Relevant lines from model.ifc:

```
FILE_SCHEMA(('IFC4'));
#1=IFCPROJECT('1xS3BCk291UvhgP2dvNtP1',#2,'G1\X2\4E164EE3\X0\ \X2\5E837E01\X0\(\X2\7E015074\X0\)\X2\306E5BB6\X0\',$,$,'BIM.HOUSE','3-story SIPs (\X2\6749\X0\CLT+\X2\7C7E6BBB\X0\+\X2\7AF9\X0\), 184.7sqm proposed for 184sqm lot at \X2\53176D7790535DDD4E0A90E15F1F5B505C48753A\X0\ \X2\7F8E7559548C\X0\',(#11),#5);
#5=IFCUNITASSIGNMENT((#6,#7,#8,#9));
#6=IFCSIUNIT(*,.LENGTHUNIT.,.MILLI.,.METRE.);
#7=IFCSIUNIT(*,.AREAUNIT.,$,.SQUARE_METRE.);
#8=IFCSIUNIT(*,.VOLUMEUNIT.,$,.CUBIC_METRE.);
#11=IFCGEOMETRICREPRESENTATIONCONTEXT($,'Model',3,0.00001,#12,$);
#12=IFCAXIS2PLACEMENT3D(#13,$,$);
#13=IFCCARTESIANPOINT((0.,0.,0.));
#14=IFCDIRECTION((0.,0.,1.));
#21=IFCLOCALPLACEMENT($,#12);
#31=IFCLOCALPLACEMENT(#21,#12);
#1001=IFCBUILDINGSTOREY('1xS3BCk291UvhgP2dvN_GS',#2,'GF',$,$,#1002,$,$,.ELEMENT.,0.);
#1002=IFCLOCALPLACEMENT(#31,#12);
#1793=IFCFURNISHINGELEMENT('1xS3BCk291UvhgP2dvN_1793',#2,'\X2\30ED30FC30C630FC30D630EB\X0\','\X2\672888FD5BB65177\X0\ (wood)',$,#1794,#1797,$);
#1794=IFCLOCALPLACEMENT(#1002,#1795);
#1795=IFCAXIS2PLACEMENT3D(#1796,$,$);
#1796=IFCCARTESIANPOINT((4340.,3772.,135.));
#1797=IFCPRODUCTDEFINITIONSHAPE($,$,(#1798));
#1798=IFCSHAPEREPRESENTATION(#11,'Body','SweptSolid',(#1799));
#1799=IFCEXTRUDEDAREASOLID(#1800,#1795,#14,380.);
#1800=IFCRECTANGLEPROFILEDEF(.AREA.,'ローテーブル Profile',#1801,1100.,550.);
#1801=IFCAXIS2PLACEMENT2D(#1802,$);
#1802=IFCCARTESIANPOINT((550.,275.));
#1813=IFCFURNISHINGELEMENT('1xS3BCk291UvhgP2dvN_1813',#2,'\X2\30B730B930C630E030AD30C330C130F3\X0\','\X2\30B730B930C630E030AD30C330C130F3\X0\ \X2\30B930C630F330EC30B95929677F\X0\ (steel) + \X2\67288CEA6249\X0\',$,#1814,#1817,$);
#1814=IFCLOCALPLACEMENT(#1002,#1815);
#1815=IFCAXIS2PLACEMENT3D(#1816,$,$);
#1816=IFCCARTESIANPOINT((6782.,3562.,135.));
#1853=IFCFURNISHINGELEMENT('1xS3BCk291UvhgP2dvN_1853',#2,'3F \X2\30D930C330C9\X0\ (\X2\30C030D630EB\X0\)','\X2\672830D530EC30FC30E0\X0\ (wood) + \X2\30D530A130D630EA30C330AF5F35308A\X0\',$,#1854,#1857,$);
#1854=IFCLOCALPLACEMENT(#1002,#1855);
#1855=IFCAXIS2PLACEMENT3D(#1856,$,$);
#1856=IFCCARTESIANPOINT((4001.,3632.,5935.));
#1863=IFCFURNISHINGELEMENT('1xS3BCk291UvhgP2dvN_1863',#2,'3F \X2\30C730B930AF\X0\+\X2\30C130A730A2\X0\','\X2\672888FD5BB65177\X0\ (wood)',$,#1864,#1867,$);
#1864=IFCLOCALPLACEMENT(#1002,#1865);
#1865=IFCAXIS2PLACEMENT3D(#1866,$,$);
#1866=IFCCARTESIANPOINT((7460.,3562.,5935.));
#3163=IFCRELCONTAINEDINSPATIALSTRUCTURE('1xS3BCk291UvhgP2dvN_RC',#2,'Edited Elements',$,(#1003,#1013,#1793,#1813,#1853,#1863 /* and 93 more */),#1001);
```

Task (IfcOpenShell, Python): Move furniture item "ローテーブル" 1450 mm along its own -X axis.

```python
import ifcopenshell
import ifcopenshell.api.geometry
import ifcopenshell.util.placement
import ifcopenshell.util.unit

model = ifcopenshell.open("model.ifc")
unit_scale = ifcopenshell.util.unit.calculate_unit_scale(model)

item = model.by_guid("1xS3BCk291UvhgP2dvN_1793")
matrix = ifcopenshell.util.placement.get_local_placement(item.ObjectPlacement)
matrix[:3, 3] -= matrix[:3, 0] * 1.45 / unit_scale
ifcopenshell.api.geometry.edit_object_placement(model, product=item, matrix=matrix, is_si=False)

print(ifcopenshell.util.placement.get_local_placement(item.ObjectPlacement).round(3) + 0.0)

model.write("model_rev.ifc")
```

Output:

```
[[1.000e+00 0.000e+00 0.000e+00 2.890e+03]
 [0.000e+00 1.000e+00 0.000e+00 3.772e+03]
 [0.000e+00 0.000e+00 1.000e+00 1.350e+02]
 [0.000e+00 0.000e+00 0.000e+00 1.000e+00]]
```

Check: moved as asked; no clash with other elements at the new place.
